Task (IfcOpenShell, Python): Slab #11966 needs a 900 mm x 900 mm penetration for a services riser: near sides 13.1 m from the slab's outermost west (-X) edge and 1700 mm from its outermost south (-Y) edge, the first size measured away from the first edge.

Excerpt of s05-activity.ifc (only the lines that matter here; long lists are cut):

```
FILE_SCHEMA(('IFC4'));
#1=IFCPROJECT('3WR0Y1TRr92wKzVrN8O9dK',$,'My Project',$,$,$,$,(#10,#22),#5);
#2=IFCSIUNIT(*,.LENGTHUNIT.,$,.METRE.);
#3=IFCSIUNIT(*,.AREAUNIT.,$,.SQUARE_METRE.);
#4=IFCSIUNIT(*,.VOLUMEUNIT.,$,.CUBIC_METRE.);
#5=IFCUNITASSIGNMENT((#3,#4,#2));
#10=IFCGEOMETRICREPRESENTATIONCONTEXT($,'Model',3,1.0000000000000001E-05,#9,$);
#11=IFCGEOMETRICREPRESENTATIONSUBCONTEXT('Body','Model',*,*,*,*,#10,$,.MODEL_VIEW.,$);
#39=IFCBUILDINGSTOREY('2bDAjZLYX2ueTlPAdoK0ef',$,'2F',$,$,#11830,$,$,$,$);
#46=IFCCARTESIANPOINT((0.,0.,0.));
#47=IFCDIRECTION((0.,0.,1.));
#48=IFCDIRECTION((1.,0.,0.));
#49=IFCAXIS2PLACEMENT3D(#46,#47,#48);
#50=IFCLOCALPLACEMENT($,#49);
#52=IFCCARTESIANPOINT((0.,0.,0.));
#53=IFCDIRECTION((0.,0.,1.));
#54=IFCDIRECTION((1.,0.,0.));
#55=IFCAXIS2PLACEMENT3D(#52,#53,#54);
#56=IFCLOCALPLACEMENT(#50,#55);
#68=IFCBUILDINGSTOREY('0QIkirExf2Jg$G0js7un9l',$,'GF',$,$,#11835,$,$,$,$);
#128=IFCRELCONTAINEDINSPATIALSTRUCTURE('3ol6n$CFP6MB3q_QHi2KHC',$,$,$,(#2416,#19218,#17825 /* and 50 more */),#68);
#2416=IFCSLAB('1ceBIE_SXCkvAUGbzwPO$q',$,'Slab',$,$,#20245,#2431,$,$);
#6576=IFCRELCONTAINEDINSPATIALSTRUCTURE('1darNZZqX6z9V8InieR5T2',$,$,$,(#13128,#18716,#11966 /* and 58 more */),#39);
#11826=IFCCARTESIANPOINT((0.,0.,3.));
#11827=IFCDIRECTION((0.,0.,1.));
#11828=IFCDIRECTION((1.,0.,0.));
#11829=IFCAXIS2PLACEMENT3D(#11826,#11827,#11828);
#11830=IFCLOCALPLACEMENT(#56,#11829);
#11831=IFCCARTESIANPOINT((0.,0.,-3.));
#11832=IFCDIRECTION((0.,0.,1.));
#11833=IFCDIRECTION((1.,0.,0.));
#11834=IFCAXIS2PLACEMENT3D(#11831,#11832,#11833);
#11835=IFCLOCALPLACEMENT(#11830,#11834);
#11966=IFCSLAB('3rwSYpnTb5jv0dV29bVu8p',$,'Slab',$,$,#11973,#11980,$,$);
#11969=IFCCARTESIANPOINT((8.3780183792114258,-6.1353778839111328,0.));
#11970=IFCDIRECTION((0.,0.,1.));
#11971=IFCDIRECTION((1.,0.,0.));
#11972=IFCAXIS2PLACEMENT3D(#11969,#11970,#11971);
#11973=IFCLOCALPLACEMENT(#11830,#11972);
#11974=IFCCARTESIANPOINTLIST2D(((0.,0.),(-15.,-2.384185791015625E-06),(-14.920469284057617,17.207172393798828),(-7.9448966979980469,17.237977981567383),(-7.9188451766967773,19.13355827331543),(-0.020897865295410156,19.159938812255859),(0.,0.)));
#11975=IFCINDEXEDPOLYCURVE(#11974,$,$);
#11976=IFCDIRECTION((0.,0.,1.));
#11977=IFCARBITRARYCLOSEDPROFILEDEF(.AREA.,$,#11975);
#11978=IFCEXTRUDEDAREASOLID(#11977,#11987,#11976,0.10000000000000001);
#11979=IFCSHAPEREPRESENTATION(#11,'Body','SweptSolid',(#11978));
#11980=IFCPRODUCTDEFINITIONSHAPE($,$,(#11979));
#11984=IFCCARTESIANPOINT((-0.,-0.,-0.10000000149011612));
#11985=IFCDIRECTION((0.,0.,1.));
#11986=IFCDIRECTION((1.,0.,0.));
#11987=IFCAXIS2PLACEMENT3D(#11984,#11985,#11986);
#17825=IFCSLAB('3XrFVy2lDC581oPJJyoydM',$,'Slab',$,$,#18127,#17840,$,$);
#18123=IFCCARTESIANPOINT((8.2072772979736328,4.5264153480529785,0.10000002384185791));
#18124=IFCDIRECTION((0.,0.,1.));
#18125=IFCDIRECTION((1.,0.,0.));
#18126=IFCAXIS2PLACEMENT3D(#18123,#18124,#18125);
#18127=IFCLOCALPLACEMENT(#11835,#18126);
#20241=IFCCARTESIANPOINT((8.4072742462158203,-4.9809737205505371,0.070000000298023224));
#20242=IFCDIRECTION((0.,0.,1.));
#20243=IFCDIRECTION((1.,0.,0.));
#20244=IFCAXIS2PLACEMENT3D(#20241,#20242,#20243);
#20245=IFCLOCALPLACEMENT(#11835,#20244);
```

```python
import numpy as np
import ifcopenshell
import ifcopenshell.api.feature
import ifcopenshell.api.geometry
import ifcopenshell.api.root
import ifcopenshell.geom
import ifcopenshell.util.placement
import ifcopenshell.util.representation
import ifcopenshell.util.shape
import ifcopenshell.util.unit

model = ifcopenshell.open("s05-activity.ifc")
unit_scale = ifcopenshell.util.unit.calculate_unit_scale(model)
settings = ifcopenshell.geom.settings()


def volume(element):
    """Net volume in cubic metres, openings subtracted."""
    shape = ifcopenshell.geom.create_shape(settings, element)
    return ifcopenshell.util.shape.get_volume(shape.geometry)


slab = model.by_id(11966)
before = volume(slab)

# Extent in the slab's own axes, in metres. The edges named are its -X and -Y sides.
slab_shape = ifcopenshell.geom.create_shape(settings, slab)
vertices = ifcopenshell.util.shape.get_vertices(slab_shape.geometry)
x_min, y_min, bottom = vertices.min(axis=0)
top = vertices[:, 2].max()

opening = ifcopenshell.api.root.create_entity(model, ifc_class="IfcOpeningElement", name="Services riser opening", predefined_type="OPENING")
context = ifcopenshell.util.representation.get_context(model, "Model", "Body", "MODEL_VIEW")
width, depth = 0.9, 0.9
outline = [(0.0, 0.0), (width, 0.0), (width, depth), (0.0, depth), (0.0, 0.0)]
# Overshoot both faces by 50 mm so the cut is clean.
shape = ifcopenshell.api.geometry.add_slab_representation(
    model, context=context, depth=top - bottom + 0.1, polyline=outline
)
ifcopenshell.api.geometry.assign_representation(model, product=opening, representation=shape)

matrix = ifcopenshell.util.placement.get_local_placement(slab.ObjectPlacement)
matrix[:, 3] = matrix @ np.append(np.array([x_min + 13.1, y_min + 1.7, bottom - 0.05]) / unit_scale, 1.0)
ifcopenshell.api.geometry.edit_object_placement(model, product=opening, matrix=matrix, is_si=False)
ifcopenshell.api.feature.add_feature(model, feature=opening, element=slab)

after = volume(slab)

print(f"slab volume {before:.3f} -> {after:.3f} m3")

model.write("s05-activity-out.ifc")
```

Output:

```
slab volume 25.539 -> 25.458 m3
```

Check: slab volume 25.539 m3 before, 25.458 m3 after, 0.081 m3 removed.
